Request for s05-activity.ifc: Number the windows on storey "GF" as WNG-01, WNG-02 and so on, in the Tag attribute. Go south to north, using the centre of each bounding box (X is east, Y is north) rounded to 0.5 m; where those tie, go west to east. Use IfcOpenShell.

First a look at what the model holds.

```python
import ifcopenshell
import ifcopenshell.util.element
import ifcopenshell.util.placement

model = ifcopenshell.open("s05-activity.ifc")
print(model.schema)
storey = next(s for s in model.by_type("IfcBuildingStorey") if s.Name == "GF")
windows = [e for e in ifcopenshell.util.element.get_decomposition(storey) if e.is_a("IfcWindow")]
for e in sorted(windows, key=lambda e: e.id()):
    origin = ifcopenshell.util.placement.get_local_placement(e.ObjectPlacement)[:3, 3]
    print(e.id(), e.Tag, e.Name, origin.round(2) + 0.0, sep=" | ")
```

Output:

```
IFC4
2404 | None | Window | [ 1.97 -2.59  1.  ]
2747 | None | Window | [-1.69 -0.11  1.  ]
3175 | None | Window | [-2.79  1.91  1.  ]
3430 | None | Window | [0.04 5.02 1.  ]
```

```python
import ifcopenshell
import ifcopenshell.geom
import ifcopenshell.util.element
import ifcopenshell.util.shape

model = ifcopenshell.open("s05-activity.ifc")
settings = ifcopenshell.geom.settings()
settings.set("use-world-coords", True)


def centre(element):
    shape = ifcopenshell.geom.create_shape(settings, element)
    return ifcopenshell.util.shape.get_bbox_centroid(shape.geometry)


storey = next(s for s in model.by_type("IfcBuildingStorey") if s.Name == "GF")
windows = [e for e in ifcopenshell.util.element.get_decomposition(storey) if e.is_a("IfcWindow")]

# Insertion points can sit at a corner or the storey origin, so sort by the geometry (in metres).
centres = {e: centre(e) for e in windows}
windows.sort(key=lambda e: (round(centres[e][1] / 0.5), centres[e][0]))

for i, e in enumerate(windows, start=1):
    number = f"WNG-{i:02d}"
    e.Tag = number
    print(e.id(), number)

model.write("s05-activity_edited.ifc")
```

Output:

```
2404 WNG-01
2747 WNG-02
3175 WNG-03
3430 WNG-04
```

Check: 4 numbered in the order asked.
